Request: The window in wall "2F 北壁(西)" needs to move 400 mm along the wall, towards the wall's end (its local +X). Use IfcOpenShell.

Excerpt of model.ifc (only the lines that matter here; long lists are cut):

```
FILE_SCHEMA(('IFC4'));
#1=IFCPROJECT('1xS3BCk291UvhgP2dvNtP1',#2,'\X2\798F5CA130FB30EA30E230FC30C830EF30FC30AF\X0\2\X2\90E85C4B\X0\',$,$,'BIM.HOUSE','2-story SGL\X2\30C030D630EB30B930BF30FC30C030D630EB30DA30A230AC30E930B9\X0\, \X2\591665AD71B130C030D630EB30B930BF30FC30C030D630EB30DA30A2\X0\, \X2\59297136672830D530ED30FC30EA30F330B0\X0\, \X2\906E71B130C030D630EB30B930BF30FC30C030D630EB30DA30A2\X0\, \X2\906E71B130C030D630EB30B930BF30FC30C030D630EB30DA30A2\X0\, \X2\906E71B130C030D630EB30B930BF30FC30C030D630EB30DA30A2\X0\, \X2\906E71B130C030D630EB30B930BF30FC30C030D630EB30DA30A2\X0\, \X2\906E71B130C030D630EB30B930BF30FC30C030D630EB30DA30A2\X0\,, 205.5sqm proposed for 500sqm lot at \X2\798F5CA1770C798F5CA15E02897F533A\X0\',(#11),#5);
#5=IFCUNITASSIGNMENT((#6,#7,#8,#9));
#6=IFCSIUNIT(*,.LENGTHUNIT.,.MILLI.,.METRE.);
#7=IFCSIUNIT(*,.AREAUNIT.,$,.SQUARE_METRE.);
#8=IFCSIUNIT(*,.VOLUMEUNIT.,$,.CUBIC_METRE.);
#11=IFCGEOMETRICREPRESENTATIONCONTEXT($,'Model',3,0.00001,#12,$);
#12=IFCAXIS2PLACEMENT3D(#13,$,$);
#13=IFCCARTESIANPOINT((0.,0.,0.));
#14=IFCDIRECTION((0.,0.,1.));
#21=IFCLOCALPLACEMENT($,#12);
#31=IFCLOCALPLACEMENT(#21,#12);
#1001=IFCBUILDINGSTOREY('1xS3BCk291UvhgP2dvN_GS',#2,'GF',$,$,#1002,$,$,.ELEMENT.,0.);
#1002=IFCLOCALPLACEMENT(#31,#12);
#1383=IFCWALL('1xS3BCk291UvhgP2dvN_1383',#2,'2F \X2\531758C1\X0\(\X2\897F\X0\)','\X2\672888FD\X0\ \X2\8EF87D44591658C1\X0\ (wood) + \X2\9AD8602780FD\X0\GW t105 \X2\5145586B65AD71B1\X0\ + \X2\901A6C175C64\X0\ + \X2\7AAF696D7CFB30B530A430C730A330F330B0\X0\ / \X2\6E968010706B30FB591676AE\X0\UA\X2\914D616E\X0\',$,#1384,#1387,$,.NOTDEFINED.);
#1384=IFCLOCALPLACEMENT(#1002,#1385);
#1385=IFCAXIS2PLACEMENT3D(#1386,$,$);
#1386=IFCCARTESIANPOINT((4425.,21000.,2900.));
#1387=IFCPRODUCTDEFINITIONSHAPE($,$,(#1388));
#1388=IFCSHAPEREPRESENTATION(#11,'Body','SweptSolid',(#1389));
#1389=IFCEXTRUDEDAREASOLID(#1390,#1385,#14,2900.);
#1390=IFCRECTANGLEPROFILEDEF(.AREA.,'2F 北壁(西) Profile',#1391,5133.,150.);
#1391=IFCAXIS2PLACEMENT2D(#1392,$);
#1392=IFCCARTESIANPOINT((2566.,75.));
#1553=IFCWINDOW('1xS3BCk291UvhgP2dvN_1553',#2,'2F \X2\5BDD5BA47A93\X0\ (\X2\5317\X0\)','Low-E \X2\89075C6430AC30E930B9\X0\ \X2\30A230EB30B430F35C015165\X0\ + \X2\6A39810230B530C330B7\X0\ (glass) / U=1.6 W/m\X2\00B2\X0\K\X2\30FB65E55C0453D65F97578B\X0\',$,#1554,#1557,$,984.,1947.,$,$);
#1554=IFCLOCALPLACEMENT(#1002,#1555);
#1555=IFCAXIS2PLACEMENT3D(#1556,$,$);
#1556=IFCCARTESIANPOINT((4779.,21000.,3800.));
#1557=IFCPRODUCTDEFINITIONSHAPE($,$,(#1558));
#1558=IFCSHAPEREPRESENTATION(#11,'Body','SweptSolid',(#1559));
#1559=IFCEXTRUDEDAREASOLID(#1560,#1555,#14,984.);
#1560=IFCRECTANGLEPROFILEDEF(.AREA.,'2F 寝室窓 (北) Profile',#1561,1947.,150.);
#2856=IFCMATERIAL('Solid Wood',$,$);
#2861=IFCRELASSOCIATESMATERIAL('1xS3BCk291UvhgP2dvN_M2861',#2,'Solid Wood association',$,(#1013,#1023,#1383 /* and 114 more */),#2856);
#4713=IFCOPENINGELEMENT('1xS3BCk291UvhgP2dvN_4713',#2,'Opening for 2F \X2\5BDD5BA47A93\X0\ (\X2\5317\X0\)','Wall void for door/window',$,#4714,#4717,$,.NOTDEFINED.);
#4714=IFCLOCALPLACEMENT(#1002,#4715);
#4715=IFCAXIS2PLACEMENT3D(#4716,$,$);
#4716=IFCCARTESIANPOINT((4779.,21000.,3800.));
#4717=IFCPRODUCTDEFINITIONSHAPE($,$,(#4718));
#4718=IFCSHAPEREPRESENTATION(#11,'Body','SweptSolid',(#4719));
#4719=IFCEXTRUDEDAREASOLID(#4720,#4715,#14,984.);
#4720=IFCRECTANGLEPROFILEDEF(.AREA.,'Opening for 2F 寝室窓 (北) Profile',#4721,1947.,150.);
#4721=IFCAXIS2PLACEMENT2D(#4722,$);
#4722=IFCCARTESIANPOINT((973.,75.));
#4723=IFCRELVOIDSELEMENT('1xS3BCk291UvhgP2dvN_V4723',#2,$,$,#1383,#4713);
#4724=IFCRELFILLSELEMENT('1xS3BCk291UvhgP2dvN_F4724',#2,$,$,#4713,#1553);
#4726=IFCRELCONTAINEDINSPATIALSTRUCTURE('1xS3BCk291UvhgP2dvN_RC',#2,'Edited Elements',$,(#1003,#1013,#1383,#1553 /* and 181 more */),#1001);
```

```python
import ifcopenshell
import ifcopenshell.api.geometry
import ifcopenshell.util.placement

model = ifcopenshell.open("model.ifc")

window = model.by_id(1553)
opening = window.FillsVoids[0].RelatingOpeningElement
wall = opening.VoidsElements[0].RelatingBuildingElement

wall_matrix = ifcopenshell.util.placement.get_local_placement(wall.ObjectPlacement)
shift = wall_matrix[:3, 0] * 400.0
before = ifcopenshell.util.placement.get_local_placement(window.ObjectPlacement)[:3, 3].copy()

# The window is not placed relative to its opening, so move both.
for product in (opening, window):
    matrix = ifcopenshell.util.placement.get_local_placement(product.ObjectPlacement)
    matrix[:3, 3] += shift
    ifcopenshell.api.geometry.edit_object_placement(model, product=product, matrix=matrix, is_si=False)

after = ifcopenshell.util.placement.get_local_placement(window.ObjectPlacement)[:3, 3]
print("window moved by", (after - before).round(3) + 0.0)

model.write("model_updated.ifc")
```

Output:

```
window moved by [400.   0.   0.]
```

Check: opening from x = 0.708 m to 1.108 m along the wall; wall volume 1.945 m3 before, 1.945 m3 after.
